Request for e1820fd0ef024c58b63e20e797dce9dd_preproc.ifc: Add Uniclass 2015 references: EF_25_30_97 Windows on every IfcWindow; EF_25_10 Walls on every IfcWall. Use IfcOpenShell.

First a look at what the model holds.

```python
import ifcopenshell

model = ifcopenshell.open("e1820fd0ef024c58b63e20e797dce9dd_preproc.ifc")
print(model.schema)
print("classifications:", [c.Name for c in model.by_type("IfcClassification")])
for ifc_class in ("IfcDoor", "IfcRoof", "IfcStair", "IfcWall", "IfcWindow"):
    print(ifc_class, len(model.by_type(ifc_class)))
```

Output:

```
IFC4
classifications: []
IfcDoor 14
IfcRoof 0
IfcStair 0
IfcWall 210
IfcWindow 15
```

```python
import ifcopenshell
import ifcopenshell.api.classification

model = ifcopenshell.open("e1820fd0ef024c58b63e20e797dce9dd_preproc.ifc")

system = ifcopenshell.api.classification.add_classification(model, classification="Uniclass 2015")

codes = {
    "IfcWindow": ("EF_25_30_97", "Windows"),
    "IfcWall": ("EF_25_10", "Walls"),
}
for ifc_class, (code, name) in codes.items():
    products = model.by_type(ifc_class)
    ifcopenshell.api.classification.add_reference(
        model, products=products, classification=system, identification=code, name=name
    )
    print(code, len(products))

model.write("e1820fd0ef024c58b63e20e797dce9dd_preproc_updated.ifc")
```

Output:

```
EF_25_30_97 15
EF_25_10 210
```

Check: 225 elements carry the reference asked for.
